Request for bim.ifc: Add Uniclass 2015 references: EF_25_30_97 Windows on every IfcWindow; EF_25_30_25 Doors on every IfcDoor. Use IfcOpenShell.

First a look at what the model holds.

```python
import ifcopenshell

model = ifcopenshell.open("bim.ifc")
print(model.schema)
print("classifications:", [c.Name for c in model.by_type("IfcClassification")])
for ifc_class in ("IfcDoor", "IfcRoof", "IfcStair", "IfcWall", "IfcWindow"):
    print(ifc_class, len(model.by_type(ifc_class)))
```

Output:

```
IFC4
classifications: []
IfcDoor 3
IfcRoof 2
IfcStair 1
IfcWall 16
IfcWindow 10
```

```python
import ifcopenshell
import ifcopenshell.api.classification

model = ifcopenshell.open("bim.ifc")

system = ifcopenshell.api.classification.add_classification(model, classification="Uniclass 2015")

codes = {
    "IfcWindow": ("EF_25_30_97", "Windows"),
    "IfcDoor": ("EF_25_30_25", "Doors"),
}
for ifc_class, (code, name) in codes.items():
    products = model.by_type(ifc_class)
    ifcopenshell.api.classification.add_reference(
        model, products=products, classification=system, identification=code, name=name
    )
    print(code, len(products))

model.write("bim_rev.ifc")
```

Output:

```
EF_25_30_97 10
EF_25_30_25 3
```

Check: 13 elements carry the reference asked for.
